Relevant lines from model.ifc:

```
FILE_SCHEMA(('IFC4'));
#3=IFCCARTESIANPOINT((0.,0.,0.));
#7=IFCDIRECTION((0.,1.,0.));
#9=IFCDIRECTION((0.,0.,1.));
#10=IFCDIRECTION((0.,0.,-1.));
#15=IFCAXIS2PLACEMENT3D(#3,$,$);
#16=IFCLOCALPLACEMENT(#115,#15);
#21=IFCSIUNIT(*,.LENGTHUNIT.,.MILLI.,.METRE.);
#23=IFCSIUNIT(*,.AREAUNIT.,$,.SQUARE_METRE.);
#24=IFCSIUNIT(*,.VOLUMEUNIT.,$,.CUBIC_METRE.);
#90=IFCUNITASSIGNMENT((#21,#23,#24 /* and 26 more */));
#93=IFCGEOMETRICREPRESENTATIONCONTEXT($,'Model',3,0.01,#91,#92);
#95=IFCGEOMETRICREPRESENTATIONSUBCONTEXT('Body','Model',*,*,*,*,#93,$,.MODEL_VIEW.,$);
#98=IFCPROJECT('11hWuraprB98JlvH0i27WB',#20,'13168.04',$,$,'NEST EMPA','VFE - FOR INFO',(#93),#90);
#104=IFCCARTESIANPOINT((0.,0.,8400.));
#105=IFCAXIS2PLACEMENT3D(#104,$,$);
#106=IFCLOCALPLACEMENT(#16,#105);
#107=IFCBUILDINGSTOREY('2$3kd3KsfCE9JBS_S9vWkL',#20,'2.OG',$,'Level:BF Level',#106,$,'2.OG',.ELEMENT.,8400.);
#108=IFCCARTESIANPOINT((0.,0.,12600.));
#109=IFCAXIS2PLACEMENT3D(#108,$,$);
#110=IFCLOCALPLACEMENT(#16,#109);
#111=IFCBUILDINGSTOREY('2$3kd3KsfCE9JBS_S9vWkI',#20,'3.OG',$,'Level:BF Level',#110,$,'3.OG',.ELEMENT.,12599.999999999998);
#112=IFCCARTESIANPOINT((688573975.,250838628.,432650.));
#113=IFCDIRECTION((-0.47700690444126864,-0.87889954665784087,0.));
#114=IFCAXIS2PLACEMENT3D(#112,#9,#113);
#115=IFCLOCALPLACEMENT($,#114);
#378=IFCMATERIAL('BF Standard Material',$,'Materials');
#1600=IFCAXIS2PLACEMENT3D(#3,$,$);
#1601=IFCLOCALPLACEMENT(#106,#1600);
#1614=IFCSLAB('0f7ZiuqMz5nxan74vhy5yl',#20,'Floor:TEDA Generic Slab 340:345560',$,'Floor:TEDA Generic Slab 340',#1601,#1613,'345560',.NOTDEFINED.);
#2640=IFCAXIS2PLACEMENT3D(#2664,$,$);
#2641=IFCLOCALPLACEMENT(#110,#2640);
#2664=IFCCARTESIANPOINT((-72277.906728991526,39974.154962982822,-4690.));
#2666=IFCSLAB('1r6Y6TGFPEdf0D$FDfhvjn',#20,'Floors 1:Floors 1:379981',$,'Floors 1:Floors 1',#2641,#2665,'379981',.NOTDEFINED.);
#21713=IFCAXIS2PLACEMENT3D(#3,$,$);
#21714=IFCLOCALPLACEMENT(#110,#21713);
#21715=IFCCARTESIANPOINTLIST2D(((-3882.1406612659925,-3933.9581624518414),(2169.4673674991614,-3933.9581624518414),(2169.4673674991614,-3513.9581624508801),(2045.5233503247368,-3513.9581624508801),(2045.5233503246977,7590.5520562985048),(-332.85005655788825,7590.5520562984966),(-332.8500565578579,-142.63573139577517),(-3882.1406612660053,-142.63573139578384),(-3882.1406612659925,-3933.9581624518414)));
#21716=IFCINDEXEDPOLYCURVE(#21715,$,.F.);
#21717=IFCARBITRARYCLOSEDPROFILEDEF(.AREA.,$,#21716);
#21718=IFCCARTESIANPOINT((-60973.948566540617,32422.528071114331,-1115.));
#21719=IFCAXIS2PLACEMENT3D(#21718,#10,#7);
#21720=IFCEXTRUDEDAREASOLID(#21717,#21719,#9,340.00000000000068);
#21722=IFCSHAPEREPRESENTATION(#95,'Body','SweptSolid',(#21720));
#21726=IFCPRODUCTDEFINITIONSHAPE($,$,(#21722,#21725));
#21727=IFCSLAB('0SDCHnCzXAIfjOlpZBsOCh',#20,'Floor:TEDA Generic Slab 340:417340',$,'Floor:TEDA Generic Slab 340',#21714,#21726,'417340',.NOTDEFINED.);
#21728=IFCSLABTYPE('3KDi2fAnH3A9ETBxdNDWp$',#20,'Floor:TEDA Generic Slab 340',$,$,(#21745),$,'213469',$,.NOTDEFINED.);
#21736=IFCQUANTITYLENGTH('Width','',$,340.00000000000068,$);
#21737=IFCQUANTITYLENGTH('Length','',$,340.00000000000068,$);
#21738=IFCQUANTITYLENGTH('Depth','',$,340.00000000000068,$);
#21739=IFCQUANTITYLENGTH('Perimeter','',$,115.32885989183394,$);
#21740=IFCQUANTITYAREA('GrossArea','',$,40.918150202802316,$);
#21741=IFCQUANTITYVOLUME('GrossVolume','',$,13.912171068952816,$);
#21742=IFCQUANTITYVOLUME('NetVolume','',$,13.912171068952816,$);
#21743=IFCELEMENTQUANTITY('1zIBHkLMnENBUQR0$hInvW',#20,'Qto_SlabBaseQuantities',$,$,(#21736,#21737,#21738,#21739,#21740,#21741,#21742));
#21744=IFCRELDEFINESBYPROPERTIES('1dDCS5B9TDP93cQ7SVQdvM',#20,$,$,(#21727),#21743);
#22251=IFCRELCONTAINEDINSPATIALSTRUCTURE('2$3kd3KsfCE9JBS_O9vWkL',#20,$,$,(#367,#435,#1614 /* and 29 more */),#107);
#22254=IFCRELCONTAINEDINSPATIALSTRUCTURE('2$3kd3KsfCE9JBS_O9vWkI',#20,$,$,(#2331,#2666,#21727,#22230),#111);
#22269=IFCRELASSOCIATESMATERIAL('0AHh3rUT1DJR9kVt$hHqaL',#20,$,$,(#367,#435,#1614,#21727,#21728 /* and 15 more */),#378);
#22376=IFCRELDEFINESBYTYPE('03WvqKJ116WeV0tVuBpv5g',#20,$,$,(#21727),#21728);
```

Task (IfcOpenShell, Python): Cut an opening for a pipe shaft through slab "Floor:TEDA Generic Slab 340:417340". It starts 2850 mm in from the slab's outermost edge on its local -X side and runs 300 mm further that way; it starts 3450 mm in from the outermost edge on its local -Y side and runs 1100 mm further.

```python
import numpy as np
import ifcopenshell
import ifcopenshell.api.feature
import ifcopenshell.api.geometry
import ifcopenshell.api.pset
import ifcopenshell.api.root
import ifcopenshell.geom
import ifcopenshell.util.element
import ifcopenshell.util.placement
import ifcopenshell.util.representation
import ifcopenshell.util.shape
import ifcopenshell.util.unit

model = ifcopenshell.open("model.ifc")
unit_scale = ifcopenshell.util.unit.calculate_unit_scale(model)
volume_scale = ifcopenshell.util.unit.calculate_unit_scale(model, "VOLUMEUNIT")
settings = ifcopenshell.geom.settings()


def volume(element):
    """Net volume in cubic metres, openings subtracted."""
    shape = ifcopenshell.geom.create_shape(settings, element)
    return ifcopenshell.util.shape.get_volume(shape.geometry)


slab = model.by_id(21727)
before = volume(slab)

# Extent in the slab's own axes, in metres. The edges named are its -X and -Y sides.
slab_shape = ifcopenshell.geom.create_shape(settings, slab)
vertices = ifcopenshell.util.shape.get_vertices(slab_shape.geometry)
x_min, y_min, bottom = vertices.min(axis=0)
top = vertices[:, 2].max()

opening = ifcopenshell.api.root.create_entity(model, ifc_class="IfcOpeningElement", name="Pipe shaft opening", predefined_type="OPENING")
context = ifcopenshell.util.representation.get_context(model, "Model", "Body", "MODEL_VIEW")
width, depth = 0.3, 1.1
outline = [(0.0, 0.0), (width, 0.0), (width, depth), (0.0, depth), (0.0, 0.0)]
# Overshoot both faces by 50 mm so the cut is clean.
shape = ifcopenshell.api.geometry.add_slab_representation(
    model, context=context, depth=top - bottom + 0.1, polyline=outline
)
ifcopenshell.api.geometry.assign_representation(model, product=opening, representation=shape)

matrix = ifcopenshell.util.placement.get_local_placement(slab.ObjectPlacement)
matrix[:, 3] = matrix @ np.append(np.array([x_min + 2.85, y_min + 3.45, bottom - 0.05]) / unit_scale, 1.0)
ifcopenshell.api.geometry.edit_object_placement(model, product=opening, matrix=matrix, is_si=False)
ifcopenshell.api.feature.add_feature(model, feature=opening, element=slab)

after = volume(slab)

# Update the slab's stored quantities.
qto = model.by_id(ifcopenshell.util.element.get_pset(slab, "Qto_SlabBaseQuantities", should_inherit=False)["id"])
ifcopenshell.api.pset.edit_qto(model, qto=qto, properties={"NetVolume": after / volume_scale})

print(f"slab volume {before:.3f} -> {after:.3f} m3")

model.write("model-out.ifc")
```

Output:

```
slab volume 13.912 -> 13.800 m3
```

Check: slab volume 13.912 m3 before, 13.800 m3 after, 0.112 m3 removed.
